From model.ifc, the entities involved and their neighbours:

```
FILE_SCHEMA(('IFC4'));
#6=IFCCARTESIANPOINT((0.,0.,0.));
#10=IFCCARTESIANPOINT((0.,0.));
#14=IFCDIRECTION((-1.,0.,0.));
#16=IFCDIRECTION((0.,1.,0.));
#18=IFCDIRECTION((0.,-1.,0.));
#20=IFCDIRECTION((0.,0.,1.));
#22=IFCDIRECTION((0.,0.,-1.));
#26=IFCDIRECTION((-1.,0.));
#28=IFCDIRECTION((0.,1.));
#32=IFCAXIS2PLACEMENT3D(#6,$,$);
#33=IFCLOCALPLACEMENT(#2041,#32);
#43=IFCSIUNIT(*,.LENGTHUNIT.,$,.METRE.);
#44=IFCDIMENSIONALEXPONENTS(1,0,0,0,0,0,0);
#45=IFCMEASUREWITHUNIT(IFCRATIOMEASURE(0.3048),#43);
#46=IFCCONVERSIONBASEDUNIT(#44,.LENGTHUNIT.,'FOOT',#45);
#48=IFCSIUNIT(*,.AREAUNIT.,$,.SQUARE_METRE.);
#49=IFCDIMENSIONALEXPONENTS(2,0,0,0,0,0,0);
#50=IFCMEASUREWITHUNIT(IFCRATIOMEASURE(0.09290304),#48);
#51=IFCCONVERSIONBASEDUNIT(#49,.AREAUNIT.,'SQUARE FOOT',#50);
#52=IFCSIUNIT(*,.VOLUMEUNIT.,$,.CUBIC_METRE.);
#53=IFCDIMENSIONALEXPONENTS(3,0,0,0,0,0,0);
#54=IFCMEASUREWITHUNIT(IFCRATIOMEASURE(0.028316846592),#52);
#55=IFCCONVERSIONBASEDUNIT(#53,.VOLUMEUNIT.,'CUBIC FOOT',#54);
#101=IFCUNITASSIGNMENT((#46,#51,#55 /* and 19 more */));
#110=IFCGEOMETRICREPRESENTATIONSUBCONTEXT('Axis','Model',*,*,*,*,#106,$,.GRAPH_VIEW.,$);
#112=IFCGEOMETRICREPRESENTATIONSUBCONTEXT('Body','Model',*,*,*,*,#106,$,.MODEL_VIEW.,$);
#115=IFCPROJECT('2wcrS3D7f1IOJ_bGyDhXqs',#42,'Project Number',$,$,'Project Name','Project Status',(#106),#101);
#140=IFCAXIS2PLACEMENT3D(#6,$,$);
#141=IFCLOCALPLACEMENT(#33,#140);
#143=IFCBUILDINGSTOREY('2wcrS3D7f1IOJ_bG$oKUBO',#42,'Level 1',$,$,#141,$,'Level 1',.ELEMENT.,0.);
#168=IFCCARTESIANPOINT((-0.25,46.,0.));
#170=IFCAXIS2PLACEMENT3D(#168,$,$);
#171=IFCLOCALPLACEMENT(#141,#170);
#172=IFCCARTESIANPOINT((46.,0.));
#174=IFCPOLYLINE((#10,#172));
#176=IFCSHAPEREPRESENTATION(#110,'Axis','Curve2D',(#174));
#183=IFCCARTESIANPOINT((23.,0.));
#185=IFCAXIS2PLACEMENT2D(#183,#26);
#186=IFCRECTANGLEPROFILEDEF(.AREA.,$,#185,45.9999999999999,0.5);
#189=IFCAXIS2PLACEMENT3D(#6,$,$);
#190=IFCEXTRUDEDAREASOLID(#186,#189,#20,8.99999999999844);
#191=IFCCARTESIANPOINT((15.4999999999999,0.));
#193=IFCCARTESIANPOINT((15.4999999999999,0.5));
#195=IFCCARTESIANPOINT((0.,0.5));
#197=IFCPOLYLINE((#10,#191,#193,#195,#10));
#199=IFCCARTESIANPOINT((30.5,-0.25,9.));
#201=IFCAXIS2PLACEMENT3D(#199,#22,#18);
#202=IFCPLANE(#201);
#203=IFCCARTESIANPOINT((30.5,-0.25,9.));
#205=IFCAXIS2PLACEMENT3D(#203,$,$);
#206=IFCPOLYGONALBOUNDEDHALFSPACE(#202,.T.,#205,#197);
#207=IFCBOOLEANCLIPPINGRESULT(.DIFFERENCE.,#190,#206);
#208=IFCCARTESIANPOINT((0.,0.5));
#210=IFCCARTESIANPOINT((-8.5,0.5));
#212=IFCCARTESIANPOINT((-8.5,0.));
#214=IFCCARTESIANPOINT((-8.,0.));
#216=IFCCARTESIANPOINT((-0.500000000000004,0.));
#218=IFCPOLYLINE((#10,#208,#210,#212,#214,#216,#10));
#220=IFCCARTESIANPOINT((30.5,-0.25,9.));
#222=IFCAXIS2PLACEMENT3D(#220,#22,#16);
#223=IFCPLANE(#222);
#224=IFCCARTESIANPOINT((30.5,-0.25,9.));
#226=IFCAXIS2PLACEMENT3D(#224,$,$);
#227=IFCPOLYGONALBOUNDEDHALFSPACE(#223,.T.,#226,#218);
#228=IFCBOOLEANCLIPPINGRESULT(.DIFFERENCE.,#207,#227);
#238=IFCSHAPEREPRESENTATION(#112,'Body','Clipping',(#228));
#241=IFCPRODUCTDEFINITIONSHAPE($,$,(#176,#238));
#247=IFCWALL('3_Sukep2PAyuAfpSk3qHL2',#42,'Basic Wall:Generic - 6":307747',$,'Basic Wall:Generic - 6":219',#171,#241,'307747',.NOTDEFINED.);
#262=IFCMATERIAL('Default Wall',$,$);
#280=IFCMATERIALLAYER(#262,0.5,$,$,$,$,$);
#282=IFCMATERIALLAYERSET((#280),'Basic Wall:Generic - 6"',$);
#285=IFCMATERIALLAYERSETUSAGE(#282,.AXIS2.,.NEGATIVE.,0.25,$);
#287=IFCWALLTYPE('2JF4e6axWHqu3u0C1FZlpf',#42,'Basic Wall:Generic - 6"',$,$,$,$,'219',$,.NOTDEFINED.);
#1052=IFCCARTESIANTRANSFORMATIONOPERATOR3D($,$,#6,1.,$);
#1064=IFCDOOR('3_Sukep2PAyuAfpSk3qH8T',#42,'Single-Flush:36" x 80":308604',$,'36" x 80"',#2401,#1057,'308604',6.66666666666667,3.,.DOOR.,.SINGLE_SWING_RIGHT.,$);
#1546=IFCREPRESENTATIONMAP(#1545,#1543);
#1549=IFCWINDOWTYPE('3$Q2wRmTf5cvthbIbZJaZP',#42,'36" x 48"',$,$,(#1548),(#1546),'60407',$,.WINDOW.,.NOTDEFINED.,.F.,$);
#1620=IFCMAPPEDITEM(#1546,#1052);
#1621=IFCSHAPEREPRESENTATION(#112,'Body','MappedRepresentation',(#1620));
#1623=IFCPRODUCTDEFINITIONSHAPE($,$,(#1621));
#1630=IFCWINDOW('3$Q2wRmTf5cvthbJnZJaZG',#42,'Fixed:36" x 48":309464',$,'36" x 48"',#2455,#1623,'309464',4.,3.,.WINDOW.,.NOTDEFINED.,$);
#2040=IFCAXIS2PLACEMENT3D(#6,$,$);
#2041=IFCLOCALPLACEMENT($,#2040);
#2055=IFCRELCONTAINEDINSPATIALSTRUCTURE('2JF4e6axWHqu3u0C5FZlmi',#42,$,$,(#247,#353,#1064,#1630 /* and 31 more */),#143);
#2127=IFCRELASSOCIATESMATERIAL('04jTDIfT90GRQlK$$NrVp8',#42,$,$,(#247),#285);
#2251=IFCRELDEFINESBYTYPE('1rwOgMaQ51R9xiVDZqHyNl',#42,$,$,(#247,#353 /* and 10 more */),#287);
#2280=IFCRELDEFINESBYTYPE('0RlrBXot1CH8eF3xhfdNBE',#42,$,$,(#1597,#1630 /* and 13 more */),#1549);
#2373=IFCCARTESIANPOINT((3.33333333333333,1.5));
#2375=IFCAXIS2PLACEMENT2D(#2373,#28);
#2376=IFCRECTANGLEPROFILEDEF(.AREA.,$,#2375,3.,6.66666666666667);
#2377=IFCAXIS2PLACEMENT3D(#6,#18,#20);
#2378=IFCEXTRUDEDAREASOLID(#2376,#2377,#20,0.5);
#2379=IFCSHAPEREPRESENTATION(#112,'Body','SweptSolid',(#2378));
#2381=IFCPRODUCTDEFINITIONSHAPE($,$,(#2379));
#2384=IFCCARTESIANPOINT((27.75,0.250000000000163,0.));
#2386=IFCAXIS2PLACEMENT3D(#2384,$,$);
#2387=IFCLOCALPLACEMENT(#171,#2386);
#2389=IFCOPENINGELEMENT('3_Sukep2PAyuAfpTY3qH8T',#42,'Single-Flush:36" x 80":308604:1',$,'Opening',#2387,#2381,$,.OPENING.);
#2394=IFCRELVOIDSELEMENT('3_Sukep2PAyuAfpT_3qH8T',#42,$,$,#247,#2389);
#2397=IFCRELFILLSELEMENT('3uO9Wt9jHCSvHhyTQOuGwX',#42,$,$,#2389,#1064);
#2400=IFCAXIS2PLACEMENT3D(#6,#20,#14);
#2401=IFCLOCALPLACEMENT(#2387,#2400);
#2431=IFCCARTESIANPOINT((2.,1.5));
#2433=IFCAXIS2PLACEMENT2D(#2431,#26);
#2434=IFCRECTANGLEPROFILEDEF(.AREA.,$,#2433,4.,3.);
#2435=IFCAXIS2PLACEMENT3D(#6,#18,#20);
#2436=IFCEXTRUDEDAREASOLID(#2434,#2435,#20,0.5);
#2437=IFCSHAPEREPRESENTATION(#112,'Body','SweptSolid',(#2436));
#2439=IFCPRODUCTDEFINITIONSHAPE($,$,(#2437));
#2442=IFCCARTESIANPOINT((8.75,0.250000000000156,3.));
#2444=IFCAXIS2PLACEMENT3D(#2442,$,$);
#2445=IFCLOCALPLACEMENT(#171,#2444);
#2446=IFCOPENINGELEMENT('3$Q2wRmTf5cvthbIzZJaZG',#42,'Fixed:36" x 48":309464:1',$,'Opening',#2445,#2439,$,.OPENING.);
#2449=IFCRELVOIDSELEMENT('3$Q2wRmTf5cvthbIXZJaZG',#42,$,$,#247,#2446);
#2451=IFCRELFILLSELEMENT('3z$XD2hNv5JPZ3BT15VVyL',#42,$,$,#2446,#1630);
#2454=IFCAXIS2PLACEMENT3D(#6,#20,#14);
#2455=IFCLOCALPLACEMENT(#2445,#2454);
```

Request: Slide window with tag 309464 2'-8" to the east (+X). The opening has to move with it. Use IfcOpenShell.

```python
import ifcopenshell
import ifcopenshell.api.geometry
import ifcopenshell.util.placement
import ifcopenshell.util.unit

model = ifcopenshell.open("model.ifc")
unit_scale = ifcopenshell.util.unit.calculate_unit_scale(model)

window = model.by_guid("3$Q2wRmTf5cvthbJnZJaZG")
opening = window.FillsVoids[0].RelatingOpeningElement
wall = opening.VoidsElements[0].RelatingBuildingElement

wall_matrix = ifcopenshell.util.placement.get_local_placement(wall.ObjectPlacement)
shift = wall_matrix[:3, 0] * 32 * 0.0254 / unit_scale
before = ifcopenshell.util.placement.get_local_placement(window.ObjectPlacement)[:3, 3].copy()

# The window is placed relative to its opening, so it follows when the opening moves.
matrix = ifcopenshell.util.placement.get_local_placement(opening.ObjectPlacement)
matrix[:3, 3] += shift
ifcopenshell.api.geometry.edit_object_placement(
    model, product=opening, matrix=matrix, is_si=False, should_transform_children=True
)

after = ifcopenshell.util.placement.get_local_placement(window.ObjectPlacement)[:3, 3]
print("window moved by", (after - before).round(3) + 0.0)

model.write("model_edited.ifc")
```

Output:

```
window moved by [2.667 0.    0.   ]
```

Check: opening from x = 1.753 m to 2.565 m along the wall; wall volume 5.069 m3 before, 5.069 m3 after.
